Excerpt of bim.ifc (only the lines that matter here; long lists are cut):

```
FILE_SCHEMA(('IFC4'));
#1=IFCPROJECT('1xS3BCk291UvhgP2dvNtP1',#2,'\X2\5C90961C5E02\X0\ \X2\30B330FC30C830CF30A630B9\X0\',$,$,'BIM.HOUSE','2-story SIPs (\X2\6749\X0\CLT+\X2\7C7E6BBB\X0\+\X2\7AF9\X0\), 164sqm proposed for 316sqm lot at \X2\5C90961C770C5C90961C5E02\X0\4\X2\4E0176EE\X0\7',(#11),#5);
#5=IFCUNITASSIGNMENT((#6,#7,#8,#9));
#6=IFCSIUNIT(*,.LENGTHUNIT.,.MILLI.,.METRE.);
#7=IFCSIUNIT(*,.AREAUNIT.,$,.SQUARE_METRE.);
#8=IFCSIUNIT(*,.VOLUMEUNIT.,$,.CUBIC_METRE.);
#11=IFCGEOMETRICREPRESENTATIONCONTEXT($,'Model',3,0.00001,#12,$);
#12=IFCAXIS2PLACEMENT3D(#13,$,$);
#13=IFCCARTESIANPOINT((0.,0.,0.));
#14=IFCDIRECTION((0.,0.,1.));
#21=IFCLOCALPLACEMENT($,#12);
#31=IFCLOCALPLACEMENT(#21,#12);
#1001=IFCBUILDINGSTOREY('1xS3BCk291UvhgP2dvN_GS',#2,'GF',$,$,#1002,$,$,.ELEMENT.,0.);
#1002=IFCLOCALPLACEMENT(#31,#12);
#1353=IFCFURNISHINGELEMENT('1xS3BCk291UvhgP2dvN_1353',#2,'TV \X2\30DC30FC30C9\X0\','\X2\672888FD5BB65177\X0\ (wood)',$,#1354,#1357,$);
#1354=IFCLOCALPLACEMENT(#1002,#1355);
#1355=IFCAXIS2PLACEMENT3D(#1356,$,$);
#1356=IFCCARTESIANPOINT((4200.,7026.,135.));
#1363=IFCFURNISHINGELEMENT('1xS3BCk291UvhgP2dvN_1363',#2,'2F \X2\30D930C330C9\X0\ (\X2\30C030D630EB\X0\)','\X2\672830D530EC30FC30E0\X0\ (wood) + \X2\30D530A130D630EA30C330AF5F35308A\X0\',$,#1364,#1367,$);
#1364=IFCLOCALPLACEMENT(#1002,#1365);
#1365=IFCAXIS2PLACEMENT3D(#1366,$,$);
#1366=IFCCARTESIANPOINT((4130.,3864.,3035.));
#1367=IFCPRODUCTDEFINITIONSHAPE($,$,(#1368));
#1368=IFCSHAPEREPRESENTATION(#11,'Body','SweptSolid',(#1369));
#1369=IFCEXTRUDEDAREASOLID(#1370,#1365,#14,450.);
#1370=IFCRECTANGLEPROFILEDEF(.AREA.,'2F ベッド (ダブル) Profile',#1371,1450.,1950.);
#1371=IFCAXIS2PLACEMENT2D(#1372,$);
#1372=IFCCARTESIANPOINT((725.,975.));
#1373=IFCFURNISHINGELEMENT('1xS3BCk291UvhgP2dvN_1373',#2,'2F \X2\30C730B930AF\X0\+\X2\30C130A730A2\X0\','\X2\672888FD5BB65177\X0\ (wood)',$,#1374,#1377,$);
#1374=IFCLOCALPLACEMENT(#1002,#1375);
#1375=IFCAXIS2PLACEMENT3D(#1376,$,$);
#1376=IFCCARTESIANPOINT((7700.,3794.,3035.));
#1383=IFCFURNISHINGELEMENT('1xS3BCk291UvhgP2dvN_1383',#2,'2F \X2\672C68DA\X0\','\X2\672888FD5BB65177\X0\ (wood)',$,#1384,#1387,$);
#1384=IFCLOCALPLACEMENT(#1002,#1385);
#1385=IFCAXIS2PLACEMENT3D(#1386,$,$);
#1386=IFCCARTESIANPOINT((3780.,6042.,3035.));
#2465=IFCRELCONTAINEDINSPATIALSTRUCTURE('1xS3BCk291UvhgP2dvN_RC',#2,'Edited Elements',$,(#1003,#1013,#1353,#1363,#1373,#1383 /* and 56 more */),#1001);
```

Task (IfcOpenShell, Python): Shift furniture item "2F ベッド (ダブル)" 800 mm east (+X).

```python
import ifcopenshell
import ifcopenshell.api.geometry
import ifcopenshell.util.placement
import ifcopenshell.util.unit

model = ifcopenshell.open("bim.ifc")
unit_scale = ifcopenshell.util.unit.calculate_unit_scale(model)

item = model.by_guid("1xS3BCk291UvhgP2dvN_1363")
matrix = ifcopenshell.util.placement.get_local_placement(item.ObjectPlacement)
matrix[0, 3] += 0.8 / unit_scale
ifcopenshell.api.geometry.edit_object_placement(model, product=item, matrix=matrix, is_si=False)

print(ifcopenshell.util.placement.get_local_placement(item.ObjectPlacement).round(3) + 0.0)

model.write("bim_rev.ifc")
```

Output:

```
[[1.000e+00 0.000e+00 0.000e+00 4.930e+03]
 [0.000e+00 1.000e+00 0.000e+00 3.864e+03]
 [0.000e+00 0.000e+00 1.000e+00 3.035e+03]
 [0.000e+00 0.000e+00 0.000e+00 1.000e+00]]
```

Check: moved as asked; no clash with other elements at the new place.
